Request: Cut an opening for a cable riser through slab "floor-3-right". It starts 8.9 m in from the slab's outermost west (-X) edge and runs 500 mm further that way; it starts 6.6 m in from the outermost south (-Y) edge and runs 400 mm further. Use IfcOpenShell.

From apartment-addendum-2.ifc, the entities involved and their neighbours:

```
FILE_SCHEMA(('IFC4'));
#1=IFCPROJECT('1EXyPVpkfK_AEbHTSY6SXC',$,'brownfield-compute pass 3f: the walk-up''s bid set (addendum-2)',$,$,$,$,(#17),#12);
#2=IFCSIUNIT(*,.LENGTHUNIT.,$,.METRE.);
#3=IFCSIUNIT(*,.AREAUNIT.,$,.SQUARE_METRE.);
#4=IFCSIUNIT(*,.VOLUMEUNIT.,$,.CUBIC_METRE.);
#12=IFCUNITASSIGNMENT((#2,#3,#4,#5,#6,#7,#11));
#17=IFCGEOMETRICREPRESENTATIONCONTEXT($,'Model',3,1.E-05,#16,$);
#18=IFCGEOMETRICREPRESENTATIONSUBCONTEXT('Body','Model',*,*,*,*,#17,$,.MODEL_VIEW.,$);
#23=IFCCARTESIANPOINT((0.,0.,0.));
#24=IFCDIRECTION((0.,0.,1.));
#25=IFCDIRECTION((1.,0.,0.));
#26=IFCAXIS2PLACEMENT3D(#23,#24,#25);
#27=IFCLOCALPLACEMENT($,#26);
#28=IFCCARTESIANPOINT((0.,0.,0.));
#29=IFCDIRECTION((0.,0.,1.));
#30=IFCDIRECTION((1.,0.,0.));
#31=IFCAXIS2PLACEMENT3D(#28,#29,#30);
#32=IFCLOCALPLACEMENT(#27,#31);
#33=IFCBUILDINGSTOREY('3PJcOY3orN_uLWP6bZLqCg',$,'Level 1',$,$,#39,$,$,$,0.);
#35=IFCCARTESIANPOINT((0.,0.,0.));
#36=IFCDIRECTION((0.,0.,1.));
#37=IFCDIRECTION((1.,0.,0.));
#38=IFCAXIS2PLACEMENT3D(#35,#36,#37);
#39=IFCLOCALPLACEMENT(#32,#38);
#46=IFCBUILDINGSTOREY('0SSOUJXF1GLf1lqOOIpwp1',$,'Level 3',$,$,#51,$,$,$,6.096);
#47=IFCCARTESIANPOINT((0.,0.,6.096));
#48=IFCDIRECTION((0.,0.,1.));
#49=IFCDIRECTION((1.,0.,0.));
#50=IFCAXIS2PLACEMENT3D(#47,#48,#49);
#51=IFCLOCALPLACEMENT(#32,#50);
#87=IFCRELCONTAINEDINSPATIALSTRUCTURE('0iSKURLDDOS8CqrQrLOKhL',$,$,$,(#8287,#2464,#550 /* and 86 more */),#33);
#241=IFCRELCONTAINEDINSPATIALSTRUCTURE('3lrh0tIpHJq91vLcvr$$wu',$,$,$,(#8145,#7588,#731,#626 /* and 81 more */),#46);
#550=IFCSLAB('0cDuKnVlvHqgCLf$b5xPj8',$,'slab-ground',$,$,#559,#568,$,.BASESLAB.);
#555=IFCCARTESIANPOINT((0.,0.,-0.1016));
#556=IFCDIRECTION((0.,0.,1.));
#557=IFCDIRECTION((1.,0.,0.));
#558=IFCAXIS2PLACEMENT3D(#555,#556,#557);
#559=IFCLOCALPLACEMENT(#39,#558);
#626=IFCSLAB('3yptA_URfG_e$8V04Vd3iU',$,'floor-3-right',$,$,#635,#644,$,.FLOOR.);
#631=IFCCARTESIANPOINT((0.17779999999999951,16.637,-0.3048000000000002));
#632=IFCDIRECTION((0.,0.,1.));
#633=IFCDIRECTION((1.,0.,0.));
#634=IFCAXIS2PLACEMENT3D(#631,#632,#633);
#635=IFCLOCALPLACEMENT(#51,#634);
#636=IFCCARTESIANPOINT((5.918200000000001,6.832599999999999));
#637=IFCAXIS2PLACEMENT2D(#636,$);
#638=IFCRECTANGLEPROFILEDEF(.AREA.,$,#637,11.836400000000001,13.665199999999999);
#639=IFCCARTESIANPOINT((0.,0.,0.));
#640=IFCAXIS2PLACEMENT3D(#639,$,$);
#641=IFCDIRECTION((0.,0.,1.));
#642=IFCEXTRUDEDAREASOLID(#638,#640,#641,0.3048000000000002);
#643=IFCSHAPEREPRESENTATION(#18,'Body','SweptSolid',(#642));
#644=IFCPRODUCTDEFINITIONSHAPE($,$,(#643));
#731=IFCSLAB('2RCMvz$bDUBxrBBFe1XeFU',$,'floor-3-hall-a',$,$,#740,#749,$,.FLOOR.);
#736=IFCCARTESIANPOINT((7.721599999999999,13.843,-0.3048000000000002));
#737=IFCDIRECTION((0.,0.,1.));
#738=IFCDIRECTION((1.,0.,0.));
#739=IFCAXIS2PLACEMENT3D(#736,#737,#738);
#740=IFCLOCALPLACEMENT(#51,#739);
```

```python
import numpy as np
import ifcopenshell
import ifcopenshell.api.feature
import ifcopenshell.api.geometry
import ifcopenshell.api.root
import ifcopenshell.geom
import ifcopenshell.util.placement
import ifcopenshell.util.representation
import ifcopenshell.util.shape
import ifcopenshell.util.unit

model = ifcopenshell.open("apartment-addendum-2.ifc")
unit_scale = ifcopenshell.util.unit.calculate_unit_scale(model)
settings = ifcopenshell.geom.settings()


def volume(element):
    """Net volume in cubic metres, openings subtracted."""
    shape = ifcopenshell.geom.create_shape(settings, element)
    return ifcopenshell.util.shape.get_volume(shape.geometry)


slab = model.by_guid("3yptA_URfG_e$8V04Vd3iU")
before = volume(slab)

# Extent in the slab's own axes, in metres. The edges named are its -X and -Y sides.
slab_shape = ifcopenshell.geom.create_shape(settings, slab)
vertices = ifcopenshell.util.shape.get_vertices(slab_shape.geometry)
x_min, y_min, bottom = vertices.min(axis=0)
top = vertices[:, 2].max()

opening = ifcopenshell.api.root.create_entity(model, ifc_class="IfcOpeningElement", name="Cable riser opening", predefined_type="OPENING")
context = ifcopenshell.util.representation.get_context(model, "Model", "Body", "MODEL_VIEW")
width, depth = 0.5, 0.4
outline = [(0.0, 0.0), (width, 0.0), (width, depth), (0.0, depth), (0.0, 0.0)]
# Overshoot both faces by 50 mm so the cut is clean.
shape = ifcopenshell.api.geometry.add_slab_representation(
    model, context=context, depth=top - bottom + 0.1, polyline=outline
)
ifcopenshell.api.geometry.assign_representation(model, product=opening, representation=shape)

matrix = ifcopenshell.util.placement.get_local_placement(slab.ObjectPlacement)
matrix[:, 3] = matrix @ np.append(np.array([x_min + 8.9, y_min + 6.6, bottom - 0.05]) / unit_scale, 1.0)
ifcopenshell.api.geometry.edit_object_placement(model, product=opening, matrix=matrix, is_si=False)
ifcopenshell.api.feature.add_feature(model, feature=opening, element=slab)

after = volume(slab)

print(f"slab volume {before:.3f} -> {after:.3f} m3")

model.write("apartment-addendum-2_edited.ifc")
```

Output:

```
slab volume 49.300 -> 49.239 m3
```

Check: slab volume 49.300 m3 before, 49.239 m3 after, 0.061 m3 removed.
